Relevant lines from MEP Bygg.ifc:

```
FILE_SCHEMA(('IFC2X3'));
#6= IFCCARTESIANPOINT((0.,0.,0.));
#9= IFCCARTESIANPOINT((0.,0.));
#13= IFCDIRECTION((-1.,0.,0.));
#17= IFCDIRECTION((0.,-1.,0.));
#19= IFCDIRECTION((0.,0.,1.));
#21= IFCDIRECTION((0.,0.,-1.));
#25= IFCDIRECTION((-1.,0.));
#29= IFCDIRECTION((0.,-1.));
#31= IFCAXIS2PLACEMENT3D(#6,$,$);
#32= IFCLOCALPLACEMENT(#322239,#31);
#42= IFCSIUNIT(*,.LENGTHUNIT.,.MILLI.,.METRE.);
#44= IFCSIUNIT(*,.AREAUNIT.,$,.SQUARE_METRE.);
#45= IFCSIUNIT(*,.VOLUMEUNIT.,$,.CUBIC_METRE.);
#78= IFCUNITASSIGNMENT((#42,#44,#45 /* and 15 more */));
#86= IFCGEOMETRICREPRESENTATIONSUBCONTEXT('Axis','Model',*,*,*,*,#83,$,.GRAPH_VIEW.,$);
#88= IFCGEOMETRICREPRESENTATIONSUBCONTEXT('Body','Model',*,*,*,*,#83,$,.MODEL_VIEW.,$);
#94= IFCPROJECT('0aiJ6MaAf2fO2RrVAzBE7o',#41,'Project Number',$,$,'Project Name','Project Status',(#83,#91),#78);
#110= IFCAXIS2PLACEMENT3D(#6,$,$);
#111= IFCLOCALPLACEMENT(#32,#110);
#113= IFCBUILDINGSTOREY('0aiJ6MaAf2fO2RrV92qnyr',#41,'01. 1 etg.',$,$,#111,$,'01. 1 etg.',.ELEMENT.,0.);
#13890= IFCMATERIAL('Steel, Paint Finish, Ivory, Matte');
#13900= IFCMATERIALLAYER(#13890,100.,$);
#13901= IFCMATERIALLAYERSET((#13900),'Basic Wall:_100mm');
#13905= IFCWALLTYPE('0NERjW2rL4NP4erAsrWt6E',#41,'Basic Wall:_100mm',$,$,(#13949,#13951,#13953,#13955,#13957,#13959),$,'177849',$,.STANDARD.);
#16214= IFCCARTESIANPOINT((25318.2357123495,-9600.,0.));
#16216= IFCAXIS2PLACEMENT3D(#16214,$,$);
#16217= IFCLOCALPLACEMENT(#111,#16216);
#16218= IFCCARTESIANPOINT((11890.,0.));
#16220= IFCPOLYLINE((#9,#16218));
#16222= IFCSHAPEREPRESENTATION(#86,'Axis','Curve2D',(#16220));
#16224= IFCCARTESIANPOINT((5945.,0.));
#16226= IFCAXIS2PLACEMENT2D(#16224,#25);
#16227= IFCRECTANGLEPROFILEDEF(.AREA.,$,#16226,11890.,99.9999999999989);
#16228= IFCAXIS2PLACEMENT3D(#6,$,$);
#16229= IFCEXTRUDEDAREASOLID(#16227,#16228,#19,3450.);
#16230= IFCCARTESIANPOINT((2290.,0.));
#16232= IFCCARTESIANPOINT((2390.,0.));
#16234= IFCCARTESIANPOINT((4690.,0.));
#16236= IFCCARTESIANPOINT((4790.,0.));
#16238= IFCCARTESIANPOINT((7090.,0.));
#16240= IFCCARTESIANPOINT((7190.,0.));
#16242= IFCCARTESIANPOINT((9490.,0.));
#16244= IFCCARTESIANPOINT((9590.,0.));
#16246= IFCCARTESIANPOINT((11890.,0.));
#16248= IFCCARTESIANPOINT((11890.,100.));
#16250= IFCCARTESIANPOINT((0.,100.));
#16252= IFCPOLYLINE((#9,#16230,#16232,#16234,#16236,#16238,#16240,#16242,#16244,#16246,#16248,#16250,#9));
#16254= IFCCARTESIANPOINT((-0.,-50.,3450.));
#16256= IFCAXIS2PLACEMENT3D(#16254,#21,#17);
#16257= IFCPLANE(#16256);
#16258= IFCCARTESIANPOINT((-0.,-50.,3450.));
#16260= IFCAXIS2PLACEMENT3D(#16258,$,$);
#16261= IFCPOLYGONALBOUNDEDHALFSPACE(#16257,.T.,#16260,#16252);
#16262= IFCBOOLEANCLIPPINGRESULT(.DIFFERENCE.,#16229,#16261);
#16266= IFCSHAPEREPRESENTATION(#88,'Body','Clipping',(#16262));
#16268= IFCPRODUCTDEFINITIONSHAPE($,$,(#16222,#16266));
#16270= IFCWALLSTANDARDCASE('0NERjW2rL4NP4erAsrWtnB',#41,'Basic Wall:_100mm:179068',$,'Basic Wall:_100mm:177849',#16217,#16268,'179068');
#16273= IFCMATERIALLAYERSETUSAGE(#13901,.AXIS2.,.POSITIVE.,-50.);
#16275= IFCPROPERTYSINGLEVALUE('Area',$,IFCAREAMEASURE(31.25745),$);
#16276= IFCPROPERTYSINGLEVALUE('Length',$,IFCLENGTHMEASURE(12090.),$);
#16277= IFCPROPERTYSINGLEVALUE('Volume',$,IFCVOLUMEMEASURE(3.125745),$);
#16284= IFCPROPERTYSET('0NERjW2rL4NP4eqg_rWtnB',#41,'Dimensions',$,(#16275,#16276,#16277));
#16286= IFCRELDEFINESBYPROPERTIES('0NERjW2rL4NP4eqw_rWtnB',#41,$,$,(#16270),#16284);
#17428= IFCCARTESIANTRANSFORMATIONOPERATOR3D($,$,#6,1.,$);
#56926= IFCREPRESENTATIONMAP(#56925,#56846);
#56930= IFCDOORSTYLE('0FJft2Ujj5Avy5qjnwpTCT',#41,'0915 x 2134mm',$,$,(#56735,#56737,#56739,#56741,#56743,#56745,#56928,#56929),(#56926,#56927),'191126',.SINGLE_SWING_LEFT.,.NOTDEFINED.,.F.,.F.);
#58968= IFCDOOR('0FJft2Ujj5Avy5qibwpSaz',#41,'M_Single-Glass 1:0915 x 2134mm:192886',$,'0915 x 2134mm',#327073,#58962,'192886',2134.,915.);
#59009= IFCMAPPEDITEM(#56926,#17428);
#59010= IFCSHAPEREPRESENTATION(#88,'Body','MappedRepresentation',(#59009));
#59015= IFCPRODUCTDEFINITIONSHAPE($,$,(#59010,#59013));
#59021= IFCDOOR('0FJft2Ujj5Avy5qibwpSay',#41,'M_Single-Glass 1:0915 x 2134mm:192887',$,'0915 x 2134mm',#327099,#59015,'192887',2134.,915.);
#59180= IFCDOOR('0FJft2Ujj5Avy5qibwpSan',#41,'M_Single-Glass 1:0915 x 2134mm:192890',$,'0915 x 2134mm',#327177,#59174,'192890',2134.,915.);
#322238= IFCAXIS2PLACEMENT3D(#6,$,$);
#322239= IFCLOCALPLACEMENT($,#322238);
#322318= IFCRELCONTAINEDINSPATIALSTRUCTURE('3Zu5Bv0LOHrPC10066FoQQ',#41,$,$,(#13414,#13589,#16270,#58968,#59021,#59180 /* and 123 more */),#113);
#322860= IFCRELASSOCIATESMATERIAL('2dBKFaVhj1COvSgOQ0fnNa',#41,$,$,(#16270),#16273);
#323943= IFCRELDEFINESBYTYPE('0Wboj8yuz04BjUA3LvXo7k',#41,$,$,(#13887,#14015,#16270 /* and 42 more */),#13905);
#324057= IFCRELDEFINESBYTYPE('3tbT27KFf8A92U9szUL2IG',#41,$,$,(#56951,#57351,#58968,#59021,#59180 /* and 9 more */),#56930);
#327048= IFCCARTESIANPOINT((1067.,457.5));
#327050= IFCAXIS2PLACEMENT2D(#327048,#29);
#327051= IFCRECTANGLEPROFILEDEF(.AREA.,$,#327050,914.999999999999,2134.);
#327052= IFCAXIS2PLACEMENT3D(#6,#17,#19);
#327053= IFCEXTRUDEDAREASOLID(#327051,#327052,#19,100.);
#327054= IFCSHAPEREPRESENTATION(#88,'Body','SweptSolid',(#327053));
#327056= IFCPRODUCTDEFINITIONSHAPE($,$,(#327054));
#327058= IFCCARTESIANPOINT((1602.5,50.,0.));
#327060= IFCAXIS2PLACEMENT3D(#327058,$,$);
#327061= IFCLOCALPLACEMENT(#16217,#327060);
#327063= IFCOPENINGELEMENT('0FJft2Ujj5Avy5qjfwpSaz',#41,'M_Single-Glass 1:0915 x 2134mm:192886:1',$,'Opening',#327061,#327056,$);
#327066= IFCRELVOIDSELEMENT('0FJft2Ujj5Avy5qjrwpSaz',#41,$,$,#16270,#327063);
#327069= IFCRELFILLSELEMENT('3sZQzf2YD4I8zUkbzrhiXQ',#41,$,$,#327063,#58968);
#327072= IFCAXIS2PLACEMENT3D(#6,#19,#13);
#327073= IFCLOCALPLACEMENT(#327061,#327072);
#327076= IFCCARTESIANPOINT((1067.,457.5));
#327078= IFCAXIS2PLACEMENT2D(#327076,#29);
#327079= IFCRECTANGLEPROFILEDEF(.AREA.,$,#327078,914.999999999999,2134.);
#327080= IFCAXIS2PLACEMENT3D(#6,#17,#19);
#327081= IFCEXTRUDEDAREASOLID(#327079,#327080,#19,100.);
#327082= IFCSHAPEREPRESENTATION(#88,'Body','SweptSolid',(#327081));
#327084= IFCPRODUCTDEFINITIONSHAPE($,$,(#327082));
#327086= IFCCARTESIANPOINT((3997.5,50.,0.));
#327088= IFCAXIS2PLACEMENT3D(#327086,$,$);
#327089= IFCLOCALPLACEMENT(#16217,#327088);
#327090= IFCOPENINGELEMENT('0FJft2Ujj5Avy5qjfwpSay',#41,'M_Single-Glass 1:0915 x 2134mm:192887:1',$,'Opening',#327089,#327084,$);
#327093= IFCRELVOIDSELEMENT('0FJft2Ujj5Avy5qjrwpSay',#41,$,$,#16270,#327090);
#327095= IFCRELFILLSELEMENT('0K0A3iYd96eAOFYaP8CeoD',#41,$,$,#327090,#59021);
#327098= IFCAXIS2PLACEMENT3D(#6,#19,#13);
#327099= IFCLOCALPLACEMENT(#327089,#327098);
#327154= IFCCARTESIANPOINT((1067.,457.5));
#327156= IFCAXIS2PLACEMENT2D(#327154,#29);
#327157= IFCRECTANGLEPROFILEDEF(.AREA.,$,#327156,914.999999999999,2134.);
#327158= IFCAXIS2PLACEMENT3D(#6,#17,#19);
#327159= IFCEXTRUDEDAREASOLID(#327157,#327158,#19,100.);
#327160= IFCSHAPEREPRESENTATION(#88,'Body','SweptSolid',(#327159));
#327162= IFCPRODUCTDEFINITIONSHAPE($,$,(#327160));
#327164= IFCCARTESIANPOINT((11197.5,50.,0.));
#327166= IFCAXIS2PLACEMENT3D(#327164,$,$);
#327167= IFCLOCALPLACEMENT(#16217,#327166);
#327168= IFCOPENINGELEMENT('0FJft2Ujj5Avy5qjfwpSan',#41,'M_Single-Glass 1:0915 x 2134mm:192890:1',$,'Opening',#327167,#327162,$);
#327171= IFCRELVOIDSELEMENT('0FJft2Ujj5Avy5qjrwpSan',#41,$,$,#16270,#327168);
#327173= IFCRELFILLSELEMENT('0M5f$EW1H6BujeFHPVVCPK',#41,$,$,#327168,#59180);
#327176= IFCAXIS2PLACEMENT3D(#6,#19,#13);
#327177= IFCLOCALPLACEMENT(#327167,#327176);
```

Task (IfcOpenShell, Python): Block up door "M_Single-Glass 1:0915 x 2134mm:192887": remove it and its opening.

```python
import ifcopenshell
import ifcopenshell.api.feature
import ifcopenshell.api.pset
import ifcopenshell.api.root
import ifcopenshell.geom
import ifcopenshell.util.element
import ifcopenshell.util.shape
import ifcopenshell.util.unit

model = ifcopenshell.open("MEP Bygg.ifc")
area_scale = ifcopenshell.util.unit.calculate_unit_scale(model, "AREAUNIT")
volume_scale = ifcopenshell.util.unit.calculate_unit_scale(model, "VOLUMEUNIT")
settings = ifcopenshell.geom.settings()


def volume(element):
    """Net volume in cubic metres, openings subtracted."""
    shape = ifcopenshell.geom.create_shape(settings, element)
    return ifcopenshell.util.shape.get_volume(shape.geometry)


door = model.by_id(59021)
opening = door.FillsVoids[0].RelatingOpeningElement
wall = opening.VoidsElements[0].RelatingBuildingElement
before = volume(wall)

ifcopenshell.api.root.remove_product(model, product=door)
ifcopenshell.api.feature.remove_feature(model, feature=opening)

after = volume(wall)
thickness = 0.1  # wall thickness in metres

# Update the wall's stored quantities.
pset = model.by_id(ifcopenshell.util.element.get_pset(wall, "Dimensions", should_inherit=False)["id"])
ifcopenshell.api.pset.edit_pset(model, pset=pset, properties={
    "Area": model.create_entity("IfcAreaMeasure", after / thickness / area_scale),
    "Volume": model.create_entity("IfcVolumeMeasure", after / volume_scale),
})

print(f"wall volume {before:.3f} -> {after:.3f} m3")

model.write("MEP Bygg_rev.ifc")
```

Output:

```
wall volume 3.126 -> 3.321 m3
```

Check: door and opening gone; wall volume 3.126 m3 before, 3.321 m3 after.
